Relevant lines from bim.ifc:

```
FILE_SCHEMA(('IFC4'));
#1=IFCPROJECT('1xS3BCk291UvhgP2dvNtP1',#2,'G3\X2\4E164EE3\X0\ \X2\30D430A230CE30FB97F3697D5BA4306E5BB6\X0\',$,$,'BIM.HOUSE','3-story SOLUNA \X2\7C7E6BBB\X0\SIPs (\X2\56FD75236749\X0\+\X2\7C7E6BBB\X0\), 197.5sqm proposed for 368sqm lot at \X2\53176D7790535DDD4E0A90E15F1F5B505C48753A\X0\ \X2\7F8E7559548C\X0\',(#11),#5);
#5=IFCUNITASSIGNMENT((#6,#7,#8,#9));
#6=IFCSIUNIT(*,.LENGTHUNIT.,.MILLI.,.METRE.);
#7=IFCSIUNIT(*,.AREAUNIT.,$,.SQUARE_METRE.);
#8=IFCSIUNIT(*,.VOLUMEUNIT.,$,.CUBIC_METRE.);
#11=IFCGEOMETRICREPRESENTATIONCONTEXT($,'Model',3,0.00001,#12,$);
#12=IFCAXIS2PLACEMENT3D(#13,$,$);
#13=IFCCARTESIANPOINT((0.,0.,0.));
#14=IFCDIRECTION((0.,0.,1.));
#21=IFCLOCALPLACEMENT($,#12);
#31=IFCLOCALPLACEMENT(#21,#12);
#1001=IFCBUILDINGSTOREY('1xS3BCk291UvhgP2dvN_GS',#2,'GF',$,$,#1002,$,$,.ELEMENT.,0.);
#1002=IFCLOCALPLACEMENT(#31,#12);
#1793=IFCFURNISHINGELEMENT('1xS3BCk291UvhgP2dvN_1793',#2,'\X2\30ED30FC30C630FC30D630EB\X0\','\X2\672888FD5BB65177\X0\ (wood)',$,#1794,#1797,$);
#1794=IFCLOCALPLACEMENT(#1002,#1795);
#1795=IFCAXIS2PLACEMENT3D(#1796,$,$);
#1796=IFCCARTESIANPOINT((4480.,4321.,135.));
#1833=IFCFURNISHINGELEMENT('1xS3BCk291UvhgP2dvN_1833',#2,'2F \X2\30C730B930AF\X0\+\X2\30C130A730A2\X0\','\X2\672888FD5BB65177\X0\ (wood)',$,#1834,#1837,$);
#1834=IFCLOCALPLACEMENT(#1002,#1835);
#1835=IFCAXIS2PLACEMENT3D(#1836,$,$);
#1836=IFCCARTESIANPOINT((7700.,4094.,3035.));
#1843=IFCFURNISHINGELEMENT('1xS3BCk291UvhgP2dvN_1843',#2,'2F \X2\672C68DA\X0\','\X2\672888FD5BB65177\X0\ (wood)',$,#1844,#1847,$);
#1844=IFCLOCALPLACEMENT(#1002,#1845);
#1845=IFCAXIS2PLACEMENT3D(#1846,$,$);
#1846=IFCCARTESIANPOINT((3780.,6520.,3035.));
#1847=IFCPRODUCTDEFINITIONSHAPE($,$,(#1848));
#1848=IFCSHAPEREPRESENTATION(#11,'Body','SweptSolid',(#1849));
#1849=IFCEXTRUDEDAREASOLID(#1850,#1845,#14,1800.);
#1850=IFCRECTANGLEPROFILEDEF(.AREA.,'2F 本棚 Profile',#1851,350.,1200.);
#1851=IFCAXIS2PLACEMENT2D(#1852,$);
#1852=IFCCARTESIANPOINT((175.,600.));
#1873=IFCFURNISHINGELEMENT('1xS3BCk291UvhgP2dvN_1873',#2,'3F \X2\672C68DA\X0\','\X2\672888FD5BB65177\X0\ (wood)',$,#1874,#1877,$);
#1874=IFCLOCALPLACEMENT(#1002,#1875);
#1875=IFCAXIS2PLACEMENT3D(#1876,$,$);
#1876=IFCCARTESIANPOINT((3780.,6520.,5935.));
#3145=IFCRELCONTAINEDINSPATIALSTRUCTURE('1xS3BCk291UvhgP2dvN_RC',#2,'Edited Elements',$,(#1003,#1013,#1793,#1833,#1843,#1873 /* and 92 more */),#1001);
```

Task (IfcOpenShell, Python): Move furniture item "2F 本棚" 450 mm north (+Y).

```python
import ifcopenshell
import ifcopenshell.api.geometry
import ifcopenshell.util.placement
import ifcopenshell.util.unit

model = ifcopenshell.open("bim.ifc")
unit_scale = ifcopenshell.util.unit.calculate_unit_scale(model)

item = model.by_guid("1xS3BCk291UvhgP2dvN_1843")
matrix = ifcopenshell.util.placement.get_local_placement(item.ObjectPlacement)
matrix[1, 3] += 0.45 / unit_scale
ifcopenshell.api.geometry.edit_object_placement(model, product=item, matrix=matrix, is_si=False)

print(ifcopenshell.util.placement.get_local_placement(item.ObjectPlacement).round(3) + 0.0)

model.write("bim-out.ifc")
```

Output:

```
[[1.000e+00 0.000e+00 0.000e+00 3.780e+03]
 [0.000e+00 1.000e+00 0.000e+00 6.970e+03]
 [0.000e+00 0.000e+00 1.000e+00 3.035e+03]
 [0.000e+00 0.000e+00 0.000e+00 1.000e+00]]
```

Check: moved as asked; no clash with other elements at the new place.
